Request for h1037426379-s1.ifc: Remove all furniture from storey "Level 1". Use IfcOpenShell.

First a look at what the model holds.

```python
import ifcopenshell
import ifcopenshell.util.element

model = ifcopenshell.open("h1037426379-s1.ifc")
print(model.schema)
storey = next(s for s in model.by_type("IfcBuildingStorey") if s.Name == "Level 1")
furniture = [e for e in ifcopenshell.util.element.get_decomposition(storey) if e.is_a("IfcFurnishingElement")]
seen = {}
for e in furniture:
    element_type = ifcopenshell.util.element.get_type(e)
    name = element_type.Name if element_type not in (None, e) else None
    seen[name] = seen.get(name, 0) + 1
for name, count in sorted(seen.items(), key=str):
    print(count, "x", name)
```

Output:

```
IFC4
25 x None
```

```python
import ifcopenshell
import ifcopenshell.api.root
import ifcopenshell.util.element

model = ifcopenshell.open("h1037426379-s1.ifc")

storey = next(s for s in model.by_type("IfcBuildingStorey") if s.Name == "Level 1")
furniture = [e for e in ifcopenshell.util.element.get_decomposition(storey) if e.is_a("IfcFurnishingElement")]

for e in furniture:
    ifcopenshell.api.root.remove_product(model, product=e)
print(len(furniture), "removed")

model.write("h1037426379-s1_edited.ifc")
```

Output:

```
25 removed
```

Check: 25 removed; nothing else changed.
